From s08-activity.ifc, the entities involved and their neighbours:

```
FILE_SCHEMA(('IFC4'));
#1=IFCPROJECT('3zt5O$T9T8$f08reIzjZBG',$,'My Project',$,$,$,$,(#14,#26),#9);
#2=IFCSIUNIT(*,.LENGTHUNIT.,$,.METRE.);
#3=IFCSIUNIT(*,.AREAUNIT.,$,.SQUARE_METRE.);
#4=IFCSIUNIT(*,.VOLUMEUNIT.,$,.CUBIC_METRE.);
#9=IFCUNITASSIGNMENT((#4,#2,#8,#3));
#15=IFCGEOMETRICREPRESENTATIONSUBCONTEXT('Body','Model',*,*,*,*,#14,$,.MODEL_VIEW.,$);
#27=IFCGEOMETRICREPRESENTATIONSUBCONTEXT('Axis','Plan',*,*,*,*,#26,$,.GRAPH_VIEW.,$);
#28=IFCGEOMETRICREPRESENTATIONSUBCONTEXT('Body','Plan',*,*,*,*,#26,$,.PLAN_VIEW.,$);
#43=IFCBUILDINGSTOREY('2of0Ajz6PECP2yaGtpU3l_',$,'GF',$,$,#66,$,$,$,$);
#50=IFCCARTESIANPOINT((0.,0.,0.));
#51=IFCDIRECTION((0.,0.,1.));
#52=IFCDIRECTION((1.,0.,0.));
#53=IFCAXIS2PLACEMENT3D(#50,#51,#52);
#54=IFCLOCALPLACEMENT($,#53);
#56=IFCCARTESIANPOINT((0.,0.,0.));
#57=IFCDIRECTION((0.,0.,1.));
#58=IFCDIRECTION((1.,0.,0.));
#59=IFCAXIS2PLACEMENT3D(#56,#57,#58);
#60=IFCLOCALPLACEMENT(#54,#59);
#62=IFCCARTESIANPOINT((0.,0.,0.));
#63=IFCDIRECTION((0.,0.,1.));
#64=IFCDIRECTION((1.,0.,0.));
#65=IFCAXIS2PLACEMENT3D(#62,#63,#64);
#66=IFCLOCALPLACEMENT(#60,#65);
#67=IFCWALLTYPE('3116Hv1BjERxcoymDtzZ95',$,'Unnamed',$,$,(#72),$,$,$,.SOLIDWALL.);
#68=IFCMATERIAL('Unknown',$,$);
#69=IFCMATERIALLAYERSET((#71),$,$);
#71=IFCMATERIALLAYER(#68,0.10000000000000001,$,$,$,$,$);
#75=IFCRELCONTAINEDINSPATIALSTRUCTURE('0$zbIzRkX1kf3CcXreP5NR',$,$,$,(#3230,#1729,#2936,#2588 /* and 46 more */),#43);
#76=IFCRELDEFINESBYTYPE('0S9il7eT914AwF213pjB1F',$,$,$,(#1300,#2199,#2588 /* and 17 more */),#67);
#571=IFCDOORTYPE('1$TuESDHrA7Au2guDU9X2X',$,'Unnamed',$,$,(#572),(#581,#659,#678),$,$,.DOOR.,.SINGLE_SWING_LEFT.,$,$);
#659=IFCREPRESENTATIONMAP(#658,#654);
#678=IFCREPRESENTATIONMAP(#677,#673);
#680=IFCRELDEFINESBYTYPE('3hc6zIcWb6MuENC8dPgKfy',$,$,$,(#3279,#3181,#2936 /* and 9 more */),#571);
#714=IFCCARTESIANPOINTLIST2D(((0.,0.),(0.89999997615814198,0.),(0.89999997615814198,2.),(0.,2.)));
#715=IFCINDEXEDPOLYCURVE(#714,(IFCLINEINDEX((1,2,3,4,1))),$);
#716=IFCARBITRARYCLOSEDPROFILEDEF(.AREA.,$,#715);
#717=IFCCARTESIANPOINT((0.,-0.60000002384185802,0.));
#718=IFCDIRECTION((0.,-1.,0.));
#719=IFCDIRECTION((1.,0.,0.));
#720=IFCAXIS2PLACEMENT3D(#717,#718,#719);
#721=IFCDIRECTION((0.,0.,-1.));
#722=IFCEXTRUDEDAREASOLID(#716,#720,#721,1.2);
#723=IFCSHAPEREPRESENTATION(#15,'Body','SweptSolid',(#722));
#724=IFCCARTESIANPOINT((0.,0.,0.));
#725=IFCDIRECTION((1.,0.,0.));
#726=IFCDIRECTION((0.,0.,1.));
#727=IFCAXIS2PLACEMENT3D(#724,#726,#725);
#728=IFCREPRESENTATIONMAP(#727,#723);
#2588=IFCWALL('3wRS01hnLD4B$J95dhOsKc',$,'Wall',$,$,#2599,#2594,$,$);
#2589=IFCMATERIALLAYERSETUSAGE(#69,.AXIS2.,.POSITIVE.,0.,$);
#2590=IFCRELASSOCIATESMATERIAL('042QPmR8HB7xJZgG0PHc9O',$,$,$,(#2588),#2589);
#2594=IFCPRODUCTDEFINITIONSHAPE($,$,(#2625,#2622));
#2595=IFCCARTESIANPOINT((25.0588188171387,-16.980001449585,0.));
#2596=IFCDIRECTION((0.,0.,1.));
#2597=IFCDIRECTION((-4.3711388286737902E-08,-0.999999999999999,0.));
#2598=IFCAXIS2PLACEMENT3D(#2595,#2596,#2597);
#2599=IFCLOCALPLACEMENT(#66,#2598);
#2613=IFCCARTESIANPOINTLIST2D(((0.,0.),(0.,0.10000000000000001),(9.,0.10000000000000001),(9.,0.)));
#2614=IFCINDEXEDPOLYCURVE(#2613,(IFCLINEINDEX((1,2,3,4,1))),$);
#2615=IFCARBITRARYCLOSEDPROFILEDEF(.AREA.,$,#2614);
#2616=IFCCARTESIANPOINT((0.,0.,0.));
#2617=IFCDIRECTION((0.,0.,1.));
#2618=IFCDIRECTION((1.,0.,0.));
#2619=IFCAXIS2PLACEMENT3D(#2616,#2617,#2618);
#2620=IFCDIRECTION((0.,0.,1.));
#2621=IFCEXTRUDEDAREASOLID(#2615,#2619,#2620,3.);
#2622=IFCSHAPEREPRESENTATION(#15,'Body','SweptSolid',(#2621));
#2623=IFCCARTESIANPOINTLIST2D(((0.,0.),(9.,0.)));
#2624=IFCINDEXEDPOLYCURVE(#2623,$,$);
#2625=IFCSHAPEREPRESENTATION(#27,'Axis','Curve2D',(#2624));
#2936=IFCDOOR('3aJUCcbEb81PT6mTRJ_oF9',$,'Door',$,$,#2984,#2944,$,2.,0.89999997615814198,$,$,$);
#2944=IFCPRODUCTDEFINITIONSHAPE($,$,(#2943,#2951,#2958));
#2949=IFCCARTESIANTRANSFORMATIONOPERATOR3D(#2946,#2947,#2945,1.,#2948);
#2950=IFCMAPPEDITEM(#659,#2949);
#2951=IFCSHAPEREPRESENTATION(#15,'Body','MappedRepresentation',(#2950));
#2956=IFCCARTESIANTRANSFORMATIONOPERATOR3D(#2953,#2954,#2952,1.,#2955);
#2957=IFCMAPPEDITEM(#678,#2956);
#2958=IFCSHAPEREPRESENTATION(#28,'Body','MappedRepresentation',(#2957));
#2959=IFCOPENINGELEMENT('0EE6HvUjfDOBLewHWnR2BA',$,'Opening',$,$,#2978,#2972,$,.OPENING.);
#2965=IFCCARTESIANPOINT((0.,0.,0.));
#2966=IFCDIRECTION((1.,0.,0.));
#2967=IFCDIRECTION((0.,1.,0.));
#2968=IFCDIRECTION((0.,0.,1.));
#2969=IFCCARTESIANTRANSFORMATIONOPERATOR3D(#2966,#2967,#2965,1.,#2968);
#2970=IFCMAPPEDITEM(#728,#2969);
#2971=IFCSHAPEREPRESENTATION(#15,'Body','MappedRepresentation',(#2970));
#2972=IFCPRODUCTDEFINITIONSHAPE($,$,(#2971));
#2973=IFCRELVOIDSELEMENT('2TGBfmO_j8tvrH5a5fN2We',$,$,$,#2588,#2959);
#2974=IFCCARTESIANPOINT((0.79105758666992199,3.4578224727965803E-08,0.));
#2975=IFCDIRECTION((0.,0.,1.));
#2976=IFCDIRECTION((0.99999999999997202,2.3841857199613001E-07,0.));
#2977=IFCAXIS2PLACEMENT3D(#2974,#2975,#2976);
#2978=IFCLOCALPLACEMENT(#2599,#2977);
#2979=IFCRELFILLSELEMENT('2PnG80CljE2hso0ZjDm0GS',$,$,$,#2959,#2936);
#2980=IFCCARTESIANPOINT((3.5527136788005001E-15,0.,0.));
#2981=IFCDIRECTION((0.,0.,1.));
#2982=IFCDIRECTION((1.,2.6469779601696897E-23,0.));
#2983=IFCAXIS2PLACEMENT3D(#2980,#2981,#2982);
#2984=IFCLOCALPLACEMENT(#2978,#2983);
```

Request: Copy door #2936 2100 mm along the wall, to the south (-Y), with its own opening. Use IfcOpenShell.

```python
import ifcopenshell
import ifcopenshell.api.feature
import ifcopenshell.api.geometry
import ifcopenshell.api.root
import ifcopenshell.geom
import ifcopenshell.util.element
import ifcopenshell.util.placement
import ifcopenshell.util.shape
import ifcopenshell.util.unit

model = ifcopenshell.open("s08-activity.ifc")
unit_scale = ifcopenshell.util.unit.calculate_unit_scale(model)
settings = ifcopenshell.geom.settings()


def volume(element):
    """Net volume in cubic metres, openings subtracted."""
    shape = ifcopenshell.geom.create_shape(settings, element)
    return ifcopenshell.util.shape.get_volume(shape.geometry)


door = model.by_guid("3aJUCcbEb81PT6mTRJ_oF9")
opening = door.FillsVoids[0].RelatingOpeningElement
wall = opening.VoidsElements[0].RelatingBuildingElement
before = volume(wall)
shift = ifcopenshell.util.placement.get_local_placement(wall.ObjectPlacement)[:3, 0] * 2.1 / unit_scale

# copy_class copies the void relationship, type, container and properties, but no geometry.
new_opening = ifcopenshell.api.root.copy_class(model, product=opening)
new_opening.Representation = ifcopenshell.util.element.copy_deep(
    model, opening.Representation, exclude=["IfcGeometricRepresentationContext", "IfcRepresentationMap"]
)
new_door = ifcopenshell.api.root.copy_class(model, product=door)
new_door.Representation = ifcopenshell.util.element.copy_deep(
    model, door.Representation, exclude=["IfcGeometricRepresentationContext", "IfcRepresentationMap"]
)
ifcopenshell.api.feature.add_filling(model, opening=new_opening, element=new_door)

for old, new in ((opening, new_opening), (door, new_door)):
    matrix = ifcopenshell.util.placement.get_local_placement(old.ObjectPlacement)
    matrix[:3, 3] += shift
    ifcopenshell.api.geometry.edit_object_placement(model, product=new, matrix=matrix, is_si=False)

after = volume(wall)

print(f"wall volume {before:.3f} -> {after:.3f} m3")

model.write("s08-activity-out.ifc")
```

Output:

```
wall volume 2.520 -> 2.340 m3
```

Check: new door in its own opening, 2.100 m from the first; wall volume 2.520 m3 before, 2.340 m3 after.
